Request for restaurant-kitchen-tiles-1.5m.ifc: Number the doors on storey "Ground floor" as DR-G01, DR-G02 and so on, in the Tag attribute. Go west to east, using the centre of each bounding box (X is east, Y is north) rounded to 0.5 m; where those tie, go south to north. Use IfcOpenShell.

First a look at what the model holds.

```python
import ifcopenshell
import ifcopenshell.util.element
import ifcopenshell.util.placement

model = ifcopenshell.open("restaurant-kitchen-tiles-1.5m.ifc")
print(model.schema)
storey = next(s for s in model.by_type("IfcBuildingStorey") if s.Name == "Ground floor")
doors = [e for e in ifcopenshell.util.element.get_decomposition(storey) if e.is_a("IfcDoor")]
for e in sorted(doors, key=lambda e: e.id()):
    origin = ifcopenshell.util.placement.get_local_placement(e.ObjectPlacement)[:3, 3]
    print(e.id(), e.Tag, e.Name, origin.round(2) + 0.0, sep=" | ")
```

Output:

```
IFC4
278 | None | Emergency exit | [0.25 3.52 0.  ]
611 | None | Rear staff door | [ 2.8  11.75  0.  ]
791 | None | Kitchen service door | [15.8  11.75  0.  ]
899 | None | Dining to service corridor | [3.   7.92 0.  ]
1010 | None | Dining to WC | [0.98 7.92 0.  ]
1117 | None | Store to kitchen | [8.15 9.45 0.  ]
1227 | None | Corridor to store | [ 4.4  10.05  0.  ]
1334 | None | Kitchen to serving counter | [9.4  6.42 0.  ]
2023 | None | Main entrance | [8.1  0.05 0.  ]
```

```python
import ifcopenshell
import ifcopenshell.geom
import ifcopenshell.util.element
import ifcopenshell.util.shape

model = ifcopenshell.open("restaurant-kitchen-tiles-1.5m.ifc")
settings = ifcopenshell.geom.settings()
settings.set("use-world-coords", True)


def centre(element):
    shape = ifcopenshell.geom.create_shape(settings, element)
    return ifcopenshell.util.shape.get_bbox_centroid(shape.geometry)


storey = next(s for s in model.by_type("IfcBuildingStorey") if s.Name == "Ground floor")
doors = [e for e in ifcopenshell.util.element.get_decomposition(storey) if e.is_a("IfcDoor")]

# Insertion points can sit at a corner or the storey origin, so sort by the geometry (in metres).
centres = {e: centre(e) for e in doors}
doors.sort(key=lambda e: (round(centres[e][0] / 0.5), centres[e][1]))

for i, e in enumerate(doors, start=1):
    number = f"DR-G{i:02d}"
    e.Tag = number
    print(e.id(), number)

model.write("restaurant-kitchen-tiles-1.5m_rev.ifc")
```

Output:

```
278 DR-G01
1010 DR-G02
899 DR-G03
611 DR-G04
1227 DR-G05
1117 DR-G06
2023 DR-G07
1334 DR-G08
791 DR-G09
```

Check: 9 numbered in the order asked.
